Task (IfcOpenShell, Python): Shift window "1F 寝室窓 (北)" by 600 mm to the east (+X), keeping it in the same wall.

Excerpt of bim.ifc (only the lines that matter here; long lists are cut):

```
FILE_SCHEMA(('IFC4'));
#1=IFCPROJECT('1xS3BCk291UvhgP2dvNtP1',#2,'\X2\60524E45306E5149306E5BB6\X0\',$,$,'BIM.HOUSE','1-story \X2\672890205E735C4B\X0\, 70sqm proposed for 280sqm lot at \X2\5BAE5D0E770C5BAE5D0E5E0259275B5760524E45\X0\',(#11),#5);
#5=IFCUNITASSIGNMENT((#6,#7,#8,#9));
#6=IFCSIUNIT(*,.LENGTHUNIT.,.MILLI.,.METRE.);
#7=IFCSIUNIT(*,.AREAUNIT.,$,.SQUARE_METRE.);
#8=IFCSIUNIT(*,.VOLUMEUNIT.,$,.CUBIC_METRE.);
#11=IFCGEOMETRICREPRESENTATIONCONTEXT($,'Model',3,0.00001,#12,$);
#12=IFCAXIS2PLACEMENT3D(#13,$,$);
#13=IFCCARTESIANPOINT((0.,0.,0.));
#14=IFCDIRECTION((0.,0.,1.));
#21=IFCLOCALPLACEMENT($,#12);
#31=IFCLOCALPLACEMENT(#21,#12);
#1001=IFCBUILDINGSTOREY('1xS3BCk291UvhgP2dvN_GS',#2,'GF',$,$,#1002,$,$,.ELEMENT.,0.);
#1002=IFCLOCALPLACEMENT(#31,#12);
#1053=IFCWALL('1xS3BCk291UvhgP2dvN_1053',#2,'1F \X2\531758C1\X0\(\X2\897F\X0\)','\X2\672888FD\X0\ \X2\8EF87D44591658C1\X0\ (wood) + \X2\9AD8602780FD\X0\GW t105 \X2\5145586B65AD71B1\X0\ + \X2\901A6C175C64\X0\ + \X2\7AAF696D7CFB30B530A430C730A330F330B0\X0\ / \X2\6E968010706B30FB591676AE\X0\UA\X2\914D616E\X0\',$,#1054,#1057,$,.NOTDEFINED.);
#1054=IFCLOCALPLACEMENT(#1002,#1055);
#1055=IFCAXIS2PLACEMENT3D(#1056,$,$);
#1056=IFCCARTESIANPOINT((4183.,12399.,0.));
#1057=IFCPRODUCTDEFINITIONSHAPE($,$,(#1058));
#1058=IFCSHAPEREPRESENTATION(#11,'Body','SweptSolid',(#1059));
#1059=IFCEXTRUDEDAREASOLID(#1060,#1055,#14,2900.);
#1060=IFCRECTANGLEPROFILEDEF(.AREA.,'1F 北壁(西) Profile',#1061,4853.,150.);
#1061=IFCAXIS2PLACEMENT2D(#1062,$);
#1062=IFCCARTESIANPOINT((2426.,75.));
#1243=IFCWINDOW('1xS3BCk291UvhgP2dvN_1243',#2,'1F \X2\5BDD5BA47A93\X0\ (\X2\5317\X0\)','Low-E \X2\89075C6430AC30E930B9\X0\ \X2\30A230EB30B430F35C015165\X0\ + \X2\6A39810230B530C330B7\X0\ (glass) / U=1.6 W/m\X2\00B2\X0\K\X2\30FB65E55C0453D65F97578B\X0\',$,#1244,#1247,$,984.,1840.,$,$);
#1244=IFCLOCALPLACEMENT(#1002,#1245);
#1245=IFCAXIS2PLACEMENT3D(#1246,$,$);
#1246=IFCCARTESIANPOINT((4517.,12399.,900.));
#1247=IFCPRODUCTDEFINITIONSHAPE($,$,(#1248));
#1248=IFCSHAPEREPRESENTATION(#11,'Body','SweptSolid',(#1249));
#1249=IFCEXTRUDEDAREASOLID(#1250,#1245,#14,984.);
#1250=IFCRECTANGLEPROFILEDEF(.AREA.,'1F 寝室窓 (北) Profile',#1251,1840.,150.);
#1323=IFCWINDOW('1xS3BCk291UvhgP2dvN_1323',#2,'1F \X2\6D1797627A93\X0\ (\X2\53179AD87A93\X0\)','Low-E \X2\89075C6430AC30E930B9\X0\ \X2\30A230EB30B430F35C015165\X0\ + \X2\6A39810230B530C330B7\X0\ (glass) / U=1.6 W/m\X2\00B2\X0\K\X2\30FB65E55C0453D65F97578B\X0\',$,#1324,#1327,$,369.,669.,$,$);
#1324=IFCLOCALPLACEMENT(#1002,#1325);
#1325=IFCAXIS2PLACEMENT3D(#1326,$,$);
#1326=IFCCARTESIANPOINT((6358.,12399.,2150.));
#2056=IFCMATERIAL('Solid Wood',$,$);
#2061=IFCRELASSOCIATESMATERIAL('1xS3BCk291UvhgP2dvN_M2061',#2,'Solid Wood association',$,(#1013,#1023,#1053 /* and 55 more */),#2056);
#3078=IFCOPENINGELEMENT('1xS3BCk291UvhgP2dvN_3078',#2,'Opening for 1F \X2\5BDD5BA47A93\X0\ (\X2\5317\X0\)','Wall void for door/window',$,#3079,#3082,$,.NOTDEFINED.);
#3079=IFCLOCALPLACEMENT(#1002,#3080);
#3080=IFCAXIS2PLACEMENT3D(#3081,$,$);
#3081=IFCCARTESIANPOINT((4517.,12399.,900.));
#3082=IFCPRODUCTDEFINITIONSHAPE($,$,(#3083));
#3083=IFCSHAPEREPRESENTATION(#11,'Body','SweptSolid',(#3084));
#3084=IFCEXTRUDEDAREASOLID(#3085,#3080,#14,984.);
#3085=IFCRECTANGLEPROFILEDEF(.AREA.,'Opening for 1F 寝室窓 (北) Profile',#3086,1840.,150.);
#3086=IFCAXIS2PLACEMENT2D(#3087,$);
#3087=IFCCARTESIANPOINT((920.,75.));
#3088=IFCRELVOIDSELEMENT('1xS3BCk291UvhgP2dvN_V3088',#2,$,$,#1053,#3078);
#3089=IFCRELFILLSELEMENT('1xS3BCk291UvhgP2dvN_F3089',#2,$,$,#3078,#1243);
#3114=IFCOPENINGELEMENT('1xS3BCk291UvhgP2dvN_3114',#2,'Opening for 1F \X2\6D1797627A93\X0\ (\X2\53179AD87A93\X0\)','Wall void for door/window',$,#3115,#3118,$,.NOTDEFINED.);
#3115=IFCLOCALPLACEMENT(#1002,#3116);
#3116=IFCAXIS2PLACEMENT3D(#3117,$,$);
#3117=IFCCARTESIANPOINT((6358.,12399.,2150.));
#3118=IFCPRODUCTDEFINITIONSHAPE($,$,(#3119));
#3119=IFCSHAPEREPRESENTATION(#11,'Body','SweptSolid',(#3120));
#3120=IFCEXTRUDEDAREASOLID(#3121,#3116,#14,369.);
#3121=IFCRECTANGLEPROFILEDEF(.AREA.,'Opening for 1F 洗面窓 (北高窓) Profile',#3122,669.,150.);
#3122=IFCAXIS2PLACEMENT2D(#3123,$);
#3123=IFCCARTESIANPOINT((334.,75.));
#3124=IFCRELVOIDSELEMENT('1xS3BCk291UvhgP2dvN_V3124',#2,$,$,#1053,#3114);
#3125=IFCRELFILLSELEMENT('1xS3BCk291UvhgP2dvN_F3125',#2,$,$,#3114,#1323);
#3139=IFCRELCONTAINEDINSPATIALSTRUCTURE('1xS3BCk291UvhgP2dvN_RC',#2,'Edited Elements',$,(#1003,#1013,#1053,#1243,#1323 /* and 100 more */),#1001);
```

```python
import ifcopenshell
import ifcopenshell.api.geometry
import ifcopenshell.util.placement

model = ifcopenshell.open("bim.ifc")

window = model.by_guid("1xS3BCk291UvhgP2dvN_1243")
opening = window.FillsVoids[0].RelatingOpeningElement
wall = opening.VoidsElements[0].RelatingBuildingElement

wall_matrix = ifcopenshell.util.placement.get_local_placement(wall.ObjectPlacement)
shift = wall_matrix[:3, 0] * 600.0
before = ifcopenshell.util.placement.get_local_placement(window.ObjectPlacement)[:3, 3].copy()

# The window is not placed relative to its opening, so move both.
for product in (opening, window):
    matrix = ifcopenshell.util.placement.get_local_placement(product.ObjectPlacement)
    matrix[:3, 3] += shift
    ifcopenshell.api.geometry.edit_object_placement(model, product=product, matrix=matrix, is_si=False)

after = ifcopenshell.util.placement.get_local_placement(window.ObjectPlacement)[:3, 3]
print("window moved by", (after - before).round(3) + 0.0)

model.write("bim_rev.ifc")
```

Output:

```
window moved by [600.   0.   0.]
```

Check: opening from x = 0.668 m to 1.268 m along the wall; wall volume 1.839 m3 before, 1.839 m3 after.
